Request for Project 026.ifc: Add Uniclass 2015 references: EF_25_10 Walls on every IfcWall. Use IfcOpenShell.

First a look at what the model holds.

```python
import ifcopenshell

model = ifcopenshell.open("Project 026.ifc")
print(model.schema)
print("classifications:", [c.Name for c in model.by_type("IfcClassification")])
for ifc_class in ("IfcDoor", "IfcRoof", "IfcStair", "IfcWall", "IfcWindow"):
    print(ifc_class, len(model.by_type(ifc_class)))
```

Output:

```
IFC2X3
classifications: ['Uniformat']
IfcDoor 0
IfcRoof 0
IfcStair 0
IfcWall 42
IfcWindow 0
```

```python
import ifcopenshell
import ifcopenshell.api.classification

model = ifcopenshell.open("Project 026.ifc")

# IFC2X3 requires Source and Edition and has no link from the project to the system.
system = model.create_entity("IfcClassification", Source="NBS", Edition="2015", Name="Uniclass 2015")

codes = {
    "IfcWall": ("EF_25_10", "Walls"),
}
for ifc_class, (code, name) in codes.items():
    products = model.by_type(ifc_class)
    ifcopenshell.api.classification.add_reference(
        model, products=products, classification=system, identification=code, name=name
    )
    print(code, len(products))

model.write("Project 026_edited.ifc")
```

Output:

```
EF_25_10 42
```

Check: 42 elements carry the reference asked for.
